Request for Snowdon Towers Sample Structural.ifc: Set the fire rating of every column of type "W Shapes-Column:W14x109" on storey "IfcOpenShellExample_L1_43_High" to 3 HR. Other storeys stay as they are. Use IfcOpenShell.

First a look at what the model holds.

```python
import ifcopenshell
import ifcopenshell.util.element

model = ifcopenshell.open("Snowdon Towers Sample Structural.ifc")
print(model.schema)
storey = next(s for s in model.by_type("IfcBuildingStorey") if s.Name == "IfcOpenShellExample_L1_43_High")
columns = [e for e in ifcopenshell.util.element.get_decomposition(storey) if e.is_a("IfcColumn")]
seen = {}
for e in columns:
    element_type = ifcopenshell.util.element.get_type(e)
    key = (element_type.Name if element_type != e and element_type else None, ifcopenshell.util.element.get_pset(e, "Pset_ColumnCommon", "FireRating"))
    seen[key] = seen.get(key, 0) + 1
for (name, value), count in sorted(seen.items(), key=str):
    print(count, "x", name, "|", value)
```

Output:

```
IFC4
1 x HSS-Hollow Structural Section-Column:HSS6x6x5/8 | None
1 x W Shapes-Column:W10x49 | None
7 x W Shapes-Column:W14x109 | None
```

```python
import ifcopenshell
import ifcopenshell.api.pset
import ifcopenshell.util.element

model = ifcopenshell.open("Snowdon Towers Sample Structural.ifc")

storey = next(s for s in model.by_type("IfcBuildingStorey") if s.Name == "IfcOpenShellExample_L1_43_High")
columns = [e for e in ifcopenshell.util.element.get_decomposition(storey) if e.is_a("IfcColumn")]

count = 0
for e in columns:
    element_type = ifcopenshell.util.element.get_type(e)
    if element_type in (None, e) or element_type.Name != "W Shapes-Column:W14x109":
        continue
    # add_pset returns the element's existing set when there is one.
    pset = ifcopenshell.api.pset.add_pset(model, product=e, name="Pset_ColumnCommon")
    ifcopenshell.api.pset.edit_pset(model, pset=pset, properties={"FireRating": "3 HR"})
    count += 1

print(count, "columns updated")

model.write("Snowdon Towers Sample Structural-out.ifc")
```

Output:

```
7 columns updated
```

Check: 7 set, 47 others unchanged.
